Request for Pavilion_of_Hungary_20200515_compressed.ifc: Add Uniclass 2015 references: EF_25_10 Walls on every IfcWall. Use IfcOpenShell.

First a look at what the model holds.

```python
import ifcopenshell

model = ifcopenshell.open("Pavilion_of_Hungary_20200515_compressed.ifc")
print(model.schema)
print("classifications:", [c.Name for c in model.by_type("IfcClassification")])
for ifc_class in ("IfcDoor", "IfcRoof", "IfcStair", "IfcWall", "IfcWindow"):
    print(ifc_class, len(model.by_type(ifc_class)))
```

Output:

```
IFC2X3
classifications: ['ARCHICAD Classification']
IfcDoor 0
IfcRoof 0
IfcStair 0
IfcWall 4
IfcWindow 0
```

```python
import ifcopenshell
import ifcopenshell.api.classification

model = ifcopenshell.open("Pavilion_of_Hungary_20200515_compressed.ifc")

# IFC2X3 requires Source and Edition and has no link from the project to the system.
system = model.create_entity("IfcClassification", Source="NBS", Edition="2015", Name="Uniclass 2015")

codes = {
    "IfcWall": ("EF_25_10", "Walls"),
}
for ifc_class, (code, name) in codes.items():
    products = model.by_type(ifc_class)
    ifcopenshell.api.classification.add_reference(
        model, products=products, classification=system, identification=code, name=name
    )
    print(code, len(products))

model.write("Pavilion_of_Hungary_20200515_compressed_rev.ifc")
```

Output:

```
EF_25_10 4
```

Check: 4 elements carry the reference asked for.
